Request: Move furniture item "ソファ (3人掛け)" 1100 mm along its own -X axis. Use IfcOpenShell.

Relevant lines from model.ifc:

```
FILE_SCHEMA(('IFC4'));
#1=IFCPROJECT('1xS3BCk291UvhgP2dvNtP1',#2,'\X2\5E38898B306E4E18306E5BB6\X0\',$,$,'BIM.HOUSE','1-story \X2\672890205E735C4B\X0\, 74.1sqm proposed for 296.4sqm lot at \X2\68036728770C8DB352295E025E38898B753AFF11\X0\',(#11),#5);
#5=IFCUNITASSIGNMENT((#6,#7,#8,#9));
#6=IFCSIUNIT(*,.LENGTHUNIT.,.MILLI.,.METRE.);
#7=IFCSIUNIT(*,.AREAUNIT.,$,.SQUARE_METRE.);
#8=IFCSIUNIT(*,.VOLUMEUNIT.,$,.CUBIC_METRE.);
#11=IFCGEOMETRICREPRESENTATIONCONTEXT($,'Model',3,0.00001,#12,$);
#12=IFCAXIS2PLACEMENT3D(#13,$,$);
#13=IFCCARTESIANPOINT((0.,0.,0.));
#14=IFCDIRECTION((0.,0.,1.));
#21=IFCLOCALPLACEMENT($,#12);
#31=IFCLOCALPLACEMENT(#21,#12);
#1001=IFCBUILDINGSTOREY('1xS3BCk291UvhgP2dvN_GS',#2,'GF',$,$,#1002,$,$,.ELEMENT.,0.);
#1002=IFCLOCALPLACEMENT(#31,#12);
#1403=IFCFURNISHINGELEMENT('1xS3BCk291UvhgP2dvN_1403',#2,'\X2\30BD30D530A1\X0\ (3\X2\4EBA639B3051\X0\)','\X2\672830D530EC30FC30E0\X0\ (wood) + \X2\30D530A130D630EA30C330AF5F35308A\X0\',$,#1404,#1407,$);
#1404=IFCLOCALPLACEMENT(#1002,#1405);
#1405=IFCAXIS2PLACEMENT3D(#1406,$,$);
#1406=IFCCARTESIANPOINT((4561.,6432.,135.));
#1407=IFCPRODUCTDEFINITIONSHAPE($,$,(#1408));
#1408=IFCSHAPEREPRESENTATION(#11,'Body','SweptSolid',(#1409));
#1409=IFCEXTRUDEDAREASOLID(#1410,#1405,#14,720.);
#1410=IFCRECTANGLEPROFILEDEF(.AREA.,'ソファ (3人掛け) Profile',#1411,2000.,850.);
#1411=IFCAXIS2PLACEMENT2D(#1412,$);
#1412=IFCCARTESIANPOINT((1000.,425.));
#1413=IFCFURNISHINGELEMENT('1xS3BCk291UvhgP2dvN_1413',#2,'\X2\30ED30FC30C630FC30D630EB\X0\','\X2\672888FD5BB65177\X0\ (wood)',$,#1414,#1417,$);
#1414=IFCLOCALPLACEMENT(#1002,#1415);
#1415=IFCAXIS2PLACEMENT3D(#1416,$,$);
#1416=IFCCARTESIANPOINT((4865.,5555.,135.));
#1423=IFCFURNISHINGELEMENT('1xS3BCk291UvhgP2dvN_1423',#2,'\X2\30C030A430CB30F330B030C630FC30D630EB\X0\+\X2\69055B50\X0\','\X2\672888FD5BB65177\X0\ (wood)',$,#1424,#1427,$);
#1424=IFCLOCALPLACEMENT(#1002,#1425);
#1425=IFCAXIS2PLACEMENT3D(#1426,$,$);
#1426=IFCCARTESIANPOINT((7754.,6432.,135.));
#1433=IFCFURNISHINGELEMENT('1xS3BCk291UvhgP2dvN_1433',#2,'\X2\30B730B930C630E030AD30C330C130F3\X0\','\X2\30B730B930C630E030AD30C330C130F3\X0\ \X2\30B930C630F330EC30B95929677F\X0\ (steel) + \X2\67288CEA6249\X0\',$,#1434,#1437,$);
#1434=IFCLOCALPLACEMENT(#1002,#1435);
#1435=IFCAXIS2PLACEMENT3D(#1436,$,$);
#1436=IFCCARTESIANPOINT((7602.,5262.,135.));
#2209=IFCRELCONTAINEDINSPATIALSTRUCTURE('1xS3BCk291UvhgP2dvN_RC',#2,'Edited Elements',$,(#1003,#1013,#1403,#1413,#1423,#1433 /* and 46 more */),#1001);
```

```python
import ifcopenshell
import ifcopenshell.api.geometry
import ifcopenshell.util.placement
import ifcopenshell.util.unit

model = ifcopenshell.open("model.ifc")
unit_scale = ifcopenshell.util.unit.calculate_unit_scale(model)

item = model.by_guid("1xS3BCk291UvhgP2dvN_1403")
matrix = ifcopenshell.util.placement.get_local_placement(item.ObjectPlacement)
matrix[:3, 3] -= matrix[:3, 0] * 1.1 / unit_scale
ifcopenshell.api.geometry.edit_object_placement(model, product=item, matrix=matrix, is_si=False)

print(ifcopenshell.util.placement.get_local_placement(item.ObjectPlacement).round(3) + 0.0)

model.write("model_edited.ifc")
```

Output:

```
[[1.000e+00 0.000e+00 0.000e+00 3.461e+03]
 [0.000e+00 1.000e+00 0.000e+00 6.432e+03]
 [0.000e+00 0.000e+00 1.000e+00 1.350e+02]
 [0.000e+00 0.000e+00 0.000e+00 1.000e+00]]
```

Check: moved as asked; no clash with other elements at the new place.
